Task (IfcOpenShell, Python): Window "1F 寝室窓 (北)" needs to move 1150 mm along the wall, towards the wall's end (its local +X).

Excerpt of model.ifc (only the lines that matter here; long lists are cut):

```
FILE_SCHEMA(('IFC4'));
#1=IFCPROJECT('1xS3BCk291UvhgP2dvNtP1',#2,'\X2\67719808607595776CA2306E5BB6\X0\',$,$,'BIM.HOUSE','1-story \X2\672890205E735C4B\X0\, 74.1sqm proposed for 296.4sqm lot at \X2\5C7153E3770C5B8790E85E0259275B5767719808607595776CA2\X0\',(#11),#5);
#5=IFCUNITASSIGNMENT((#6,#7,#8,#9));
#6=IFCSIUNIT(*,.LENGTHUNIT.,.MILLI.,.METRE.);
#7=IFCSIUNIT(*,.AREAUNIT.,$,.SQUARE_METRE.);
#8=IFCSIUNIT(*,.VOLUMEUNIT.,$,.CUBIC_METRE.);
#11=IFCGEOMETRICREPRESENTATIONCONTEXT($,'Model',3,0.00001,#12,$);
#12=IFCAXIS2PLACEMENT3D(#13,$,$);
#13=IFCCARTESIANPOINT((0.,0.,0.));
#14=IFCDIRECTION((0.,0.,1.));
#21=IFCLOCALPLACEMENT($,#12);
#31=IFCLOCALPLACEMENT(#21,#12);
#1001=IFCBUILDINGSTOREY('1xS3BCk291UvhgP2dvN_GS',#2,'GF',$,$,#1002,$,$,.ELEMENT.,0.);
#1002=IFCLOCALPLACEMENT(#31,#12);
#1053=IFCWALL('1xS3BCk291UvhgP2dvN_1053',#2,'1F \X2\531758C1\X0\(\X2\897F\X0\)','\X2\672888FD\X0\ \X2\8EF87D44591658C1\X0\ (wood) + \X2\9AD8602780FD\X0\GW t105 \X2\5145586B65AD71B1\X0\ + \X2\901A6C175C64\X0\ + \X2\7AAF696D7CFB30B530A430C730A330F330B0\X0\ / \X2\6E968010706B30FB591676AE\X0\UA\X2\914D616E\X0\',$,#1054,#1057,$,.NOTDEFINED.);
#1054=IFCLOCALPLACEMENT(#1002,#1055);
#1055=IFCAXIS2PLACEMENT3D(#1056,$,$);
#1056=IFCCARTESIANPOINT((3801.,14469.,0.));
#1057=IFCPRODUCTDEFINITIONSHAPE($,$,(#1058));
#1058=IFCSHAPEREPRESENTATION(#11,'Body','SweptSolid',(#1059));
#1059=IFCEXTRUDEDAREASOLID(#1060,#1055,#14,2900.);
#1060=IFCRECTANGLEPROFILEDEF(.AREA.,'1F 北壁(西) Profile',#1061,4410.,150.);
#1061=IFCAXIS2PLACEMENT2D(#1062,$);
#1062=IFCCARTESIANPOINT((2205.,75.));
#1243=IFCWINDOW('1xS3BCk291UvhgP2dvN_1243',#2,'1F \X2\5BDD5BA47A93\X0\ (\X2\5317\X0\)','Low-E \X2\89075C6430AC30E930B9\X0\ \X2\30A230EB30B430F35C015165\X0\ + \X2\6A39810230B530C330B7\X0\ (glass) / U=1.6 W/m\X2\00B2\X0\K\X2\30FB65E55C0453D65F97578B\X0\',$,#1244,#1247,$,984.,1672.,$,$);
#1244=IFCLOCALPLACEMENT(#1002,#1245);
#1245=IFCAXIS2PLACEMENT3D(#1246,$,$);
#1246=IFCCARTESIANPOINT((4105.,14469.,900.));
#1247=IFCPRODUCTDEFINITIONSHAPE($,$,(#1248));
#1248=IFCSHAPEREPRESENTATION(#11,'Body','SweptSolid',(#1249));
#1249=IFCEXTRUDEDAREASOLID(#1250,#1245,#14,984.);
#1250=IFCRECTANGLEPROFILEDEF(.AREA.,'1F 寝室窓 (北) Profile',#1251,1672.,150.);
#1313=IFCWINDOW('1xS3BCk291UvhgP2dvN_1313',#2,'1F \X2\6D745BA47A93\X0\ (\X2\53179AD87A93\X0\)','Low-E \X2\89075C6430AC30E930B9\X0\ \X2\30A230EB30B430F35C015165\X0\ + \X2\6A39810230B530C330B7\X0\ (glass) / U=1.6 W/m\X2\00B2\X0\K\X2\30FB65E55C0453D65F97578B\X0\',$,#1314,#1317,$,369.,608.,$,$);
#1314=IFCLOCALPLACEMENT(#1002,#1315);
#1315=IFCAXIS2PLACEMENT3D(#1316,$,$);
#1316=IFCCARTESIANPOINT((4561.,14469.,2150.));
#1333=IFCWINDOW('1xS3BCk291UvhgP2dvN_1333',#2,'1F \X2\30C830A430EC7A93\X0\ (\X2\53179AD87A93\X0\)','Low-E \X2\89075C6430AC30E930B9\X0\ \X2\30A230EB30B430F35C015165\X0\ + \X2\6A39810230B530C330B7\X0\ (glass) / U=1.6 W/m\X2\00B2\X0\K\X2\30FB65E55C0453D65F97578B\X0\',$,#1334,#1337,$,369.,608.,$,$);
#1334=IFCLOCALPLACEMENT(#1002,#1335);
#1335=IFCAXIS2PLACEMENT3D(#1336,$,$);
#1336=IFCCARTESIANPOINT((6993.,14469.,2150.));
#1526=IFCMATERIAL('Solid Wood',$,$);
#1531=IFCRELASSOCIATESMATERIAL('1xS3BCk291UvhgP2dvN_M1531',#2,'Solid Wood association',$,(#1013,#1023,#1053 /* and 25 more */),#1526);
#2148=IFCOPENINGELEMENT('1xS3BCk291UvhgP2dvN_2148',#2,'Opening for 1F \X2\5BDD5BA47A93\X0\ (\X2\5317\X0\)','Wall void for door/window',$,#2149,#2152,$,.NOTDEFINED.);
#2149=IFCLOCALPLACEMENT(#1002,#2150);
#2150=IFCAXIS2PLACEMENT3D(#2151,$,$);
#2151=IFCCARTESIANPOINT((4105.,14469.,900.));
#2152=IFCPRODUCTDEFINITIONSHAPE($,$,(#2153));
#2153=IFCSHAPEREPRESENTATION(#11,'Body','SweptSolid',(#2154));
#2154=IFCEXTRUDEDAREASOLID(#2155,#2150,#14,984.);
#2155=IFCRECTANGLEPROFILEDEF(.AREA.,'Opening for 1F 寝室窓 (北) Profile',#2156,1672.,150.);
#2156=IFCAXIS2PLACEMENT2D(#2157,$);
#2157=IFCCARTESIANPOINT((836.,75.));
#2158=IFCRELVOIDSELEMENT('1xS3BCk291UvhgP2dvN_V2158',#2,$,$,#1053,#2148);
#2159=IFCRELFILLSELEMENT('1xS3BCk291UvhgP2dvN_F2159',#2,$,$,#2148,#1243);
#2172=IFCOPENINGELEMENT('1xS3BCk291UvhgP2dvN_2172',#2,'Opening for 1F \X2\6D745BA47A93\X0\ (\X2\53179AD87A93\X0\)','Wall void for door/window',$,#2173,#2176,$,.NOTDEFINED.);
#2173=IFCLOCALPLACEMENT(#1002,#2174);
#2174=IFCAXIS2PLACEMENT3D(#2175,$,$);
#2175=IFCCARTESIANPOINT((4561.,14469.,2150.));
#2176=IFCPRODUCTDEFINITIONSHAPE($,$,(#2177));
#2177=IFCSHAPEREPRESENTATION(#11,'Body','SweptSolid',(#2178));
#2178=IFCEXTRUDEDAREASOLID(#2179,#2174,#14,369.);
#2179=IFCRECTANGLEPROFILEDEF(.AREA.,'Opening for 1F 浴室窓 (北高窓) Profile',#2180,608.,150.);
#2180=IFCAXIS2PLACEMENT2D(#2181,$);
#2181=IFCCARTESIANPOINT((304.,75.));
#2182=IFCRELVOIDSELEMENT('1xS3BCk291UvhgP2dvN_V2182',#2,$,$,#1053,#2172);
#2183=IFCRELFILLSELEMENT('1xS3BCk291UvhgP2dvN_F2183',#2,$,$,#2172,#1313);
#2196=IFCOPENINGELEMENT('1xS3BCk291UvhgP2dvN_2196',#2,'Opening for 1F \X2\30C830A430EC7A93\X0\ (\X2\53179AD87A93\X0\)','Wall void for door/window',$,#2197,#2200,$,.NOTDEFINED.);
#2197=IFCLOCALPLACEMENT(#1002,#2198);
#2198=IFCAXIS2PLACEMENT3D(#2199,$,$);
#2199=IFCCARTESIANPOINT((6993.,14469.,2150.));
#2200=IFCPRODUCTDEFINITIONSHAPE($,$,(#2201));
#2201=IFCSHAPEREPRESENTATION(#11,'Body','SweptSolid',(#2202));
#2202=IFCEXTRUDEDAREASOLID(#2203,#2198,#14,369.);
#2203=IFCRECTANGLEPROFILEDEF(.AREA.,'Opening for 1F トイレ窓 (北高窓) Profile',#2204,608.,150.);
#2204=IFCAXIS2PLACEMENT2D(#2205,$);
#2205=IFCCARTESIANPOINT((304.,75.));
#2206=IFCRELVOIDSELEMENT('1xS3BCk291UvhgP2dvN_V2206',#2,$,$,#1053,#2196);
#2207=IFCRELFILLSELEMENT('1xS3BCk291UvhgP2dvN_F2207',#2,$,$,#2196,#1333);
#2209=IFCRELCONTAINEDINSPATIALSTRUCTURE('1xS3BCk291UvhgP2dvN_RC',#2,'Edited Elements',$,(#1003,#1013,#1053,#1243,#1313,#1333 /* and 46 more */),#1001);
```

```python
import ifcopenshell
import ifcopenshell.api.geometry
import ifcopenshell.util.placement

model = ifcopenshell.open("model.ifc")

window = model.by_id(1243)
opening = window.FillsVoids[0].RelatingOpeningElement
wall = opening.VoidsElements[0].RelatingBuildingElement

wall_matrix = ifcopenshell.util.placement.get_local_placement(wall.ObjectPlacement)
shift = wall_matrix[:3, 0] * 1150.0
before = ifcopenshell.util.placement.get_local_placement(window.ObjectPlacement)[:3, 3].copy()

# The window is not placed relative to its opening, so move both.
for product in (opening, window):
    matrix = ifcopenshell.util.placement.get_local_placement(product.ObjectPlacement)
    matrix[:3, 3] += shift
    ifcopenshell.api.geometry.edit_object_placement(model, product=product, matrix=matrix, is_si=False)

after = ifcopenshell.util.placement.get_local_placement(window.ObjectPlacement)[:3, 3]
print("window moved by", (after - before).round(3) + 0.0)

model.write("model_updated.ifc")
```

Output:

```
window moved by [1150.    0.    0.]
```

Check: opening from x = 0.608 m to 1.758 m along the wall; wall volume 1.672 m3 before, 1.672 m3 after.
